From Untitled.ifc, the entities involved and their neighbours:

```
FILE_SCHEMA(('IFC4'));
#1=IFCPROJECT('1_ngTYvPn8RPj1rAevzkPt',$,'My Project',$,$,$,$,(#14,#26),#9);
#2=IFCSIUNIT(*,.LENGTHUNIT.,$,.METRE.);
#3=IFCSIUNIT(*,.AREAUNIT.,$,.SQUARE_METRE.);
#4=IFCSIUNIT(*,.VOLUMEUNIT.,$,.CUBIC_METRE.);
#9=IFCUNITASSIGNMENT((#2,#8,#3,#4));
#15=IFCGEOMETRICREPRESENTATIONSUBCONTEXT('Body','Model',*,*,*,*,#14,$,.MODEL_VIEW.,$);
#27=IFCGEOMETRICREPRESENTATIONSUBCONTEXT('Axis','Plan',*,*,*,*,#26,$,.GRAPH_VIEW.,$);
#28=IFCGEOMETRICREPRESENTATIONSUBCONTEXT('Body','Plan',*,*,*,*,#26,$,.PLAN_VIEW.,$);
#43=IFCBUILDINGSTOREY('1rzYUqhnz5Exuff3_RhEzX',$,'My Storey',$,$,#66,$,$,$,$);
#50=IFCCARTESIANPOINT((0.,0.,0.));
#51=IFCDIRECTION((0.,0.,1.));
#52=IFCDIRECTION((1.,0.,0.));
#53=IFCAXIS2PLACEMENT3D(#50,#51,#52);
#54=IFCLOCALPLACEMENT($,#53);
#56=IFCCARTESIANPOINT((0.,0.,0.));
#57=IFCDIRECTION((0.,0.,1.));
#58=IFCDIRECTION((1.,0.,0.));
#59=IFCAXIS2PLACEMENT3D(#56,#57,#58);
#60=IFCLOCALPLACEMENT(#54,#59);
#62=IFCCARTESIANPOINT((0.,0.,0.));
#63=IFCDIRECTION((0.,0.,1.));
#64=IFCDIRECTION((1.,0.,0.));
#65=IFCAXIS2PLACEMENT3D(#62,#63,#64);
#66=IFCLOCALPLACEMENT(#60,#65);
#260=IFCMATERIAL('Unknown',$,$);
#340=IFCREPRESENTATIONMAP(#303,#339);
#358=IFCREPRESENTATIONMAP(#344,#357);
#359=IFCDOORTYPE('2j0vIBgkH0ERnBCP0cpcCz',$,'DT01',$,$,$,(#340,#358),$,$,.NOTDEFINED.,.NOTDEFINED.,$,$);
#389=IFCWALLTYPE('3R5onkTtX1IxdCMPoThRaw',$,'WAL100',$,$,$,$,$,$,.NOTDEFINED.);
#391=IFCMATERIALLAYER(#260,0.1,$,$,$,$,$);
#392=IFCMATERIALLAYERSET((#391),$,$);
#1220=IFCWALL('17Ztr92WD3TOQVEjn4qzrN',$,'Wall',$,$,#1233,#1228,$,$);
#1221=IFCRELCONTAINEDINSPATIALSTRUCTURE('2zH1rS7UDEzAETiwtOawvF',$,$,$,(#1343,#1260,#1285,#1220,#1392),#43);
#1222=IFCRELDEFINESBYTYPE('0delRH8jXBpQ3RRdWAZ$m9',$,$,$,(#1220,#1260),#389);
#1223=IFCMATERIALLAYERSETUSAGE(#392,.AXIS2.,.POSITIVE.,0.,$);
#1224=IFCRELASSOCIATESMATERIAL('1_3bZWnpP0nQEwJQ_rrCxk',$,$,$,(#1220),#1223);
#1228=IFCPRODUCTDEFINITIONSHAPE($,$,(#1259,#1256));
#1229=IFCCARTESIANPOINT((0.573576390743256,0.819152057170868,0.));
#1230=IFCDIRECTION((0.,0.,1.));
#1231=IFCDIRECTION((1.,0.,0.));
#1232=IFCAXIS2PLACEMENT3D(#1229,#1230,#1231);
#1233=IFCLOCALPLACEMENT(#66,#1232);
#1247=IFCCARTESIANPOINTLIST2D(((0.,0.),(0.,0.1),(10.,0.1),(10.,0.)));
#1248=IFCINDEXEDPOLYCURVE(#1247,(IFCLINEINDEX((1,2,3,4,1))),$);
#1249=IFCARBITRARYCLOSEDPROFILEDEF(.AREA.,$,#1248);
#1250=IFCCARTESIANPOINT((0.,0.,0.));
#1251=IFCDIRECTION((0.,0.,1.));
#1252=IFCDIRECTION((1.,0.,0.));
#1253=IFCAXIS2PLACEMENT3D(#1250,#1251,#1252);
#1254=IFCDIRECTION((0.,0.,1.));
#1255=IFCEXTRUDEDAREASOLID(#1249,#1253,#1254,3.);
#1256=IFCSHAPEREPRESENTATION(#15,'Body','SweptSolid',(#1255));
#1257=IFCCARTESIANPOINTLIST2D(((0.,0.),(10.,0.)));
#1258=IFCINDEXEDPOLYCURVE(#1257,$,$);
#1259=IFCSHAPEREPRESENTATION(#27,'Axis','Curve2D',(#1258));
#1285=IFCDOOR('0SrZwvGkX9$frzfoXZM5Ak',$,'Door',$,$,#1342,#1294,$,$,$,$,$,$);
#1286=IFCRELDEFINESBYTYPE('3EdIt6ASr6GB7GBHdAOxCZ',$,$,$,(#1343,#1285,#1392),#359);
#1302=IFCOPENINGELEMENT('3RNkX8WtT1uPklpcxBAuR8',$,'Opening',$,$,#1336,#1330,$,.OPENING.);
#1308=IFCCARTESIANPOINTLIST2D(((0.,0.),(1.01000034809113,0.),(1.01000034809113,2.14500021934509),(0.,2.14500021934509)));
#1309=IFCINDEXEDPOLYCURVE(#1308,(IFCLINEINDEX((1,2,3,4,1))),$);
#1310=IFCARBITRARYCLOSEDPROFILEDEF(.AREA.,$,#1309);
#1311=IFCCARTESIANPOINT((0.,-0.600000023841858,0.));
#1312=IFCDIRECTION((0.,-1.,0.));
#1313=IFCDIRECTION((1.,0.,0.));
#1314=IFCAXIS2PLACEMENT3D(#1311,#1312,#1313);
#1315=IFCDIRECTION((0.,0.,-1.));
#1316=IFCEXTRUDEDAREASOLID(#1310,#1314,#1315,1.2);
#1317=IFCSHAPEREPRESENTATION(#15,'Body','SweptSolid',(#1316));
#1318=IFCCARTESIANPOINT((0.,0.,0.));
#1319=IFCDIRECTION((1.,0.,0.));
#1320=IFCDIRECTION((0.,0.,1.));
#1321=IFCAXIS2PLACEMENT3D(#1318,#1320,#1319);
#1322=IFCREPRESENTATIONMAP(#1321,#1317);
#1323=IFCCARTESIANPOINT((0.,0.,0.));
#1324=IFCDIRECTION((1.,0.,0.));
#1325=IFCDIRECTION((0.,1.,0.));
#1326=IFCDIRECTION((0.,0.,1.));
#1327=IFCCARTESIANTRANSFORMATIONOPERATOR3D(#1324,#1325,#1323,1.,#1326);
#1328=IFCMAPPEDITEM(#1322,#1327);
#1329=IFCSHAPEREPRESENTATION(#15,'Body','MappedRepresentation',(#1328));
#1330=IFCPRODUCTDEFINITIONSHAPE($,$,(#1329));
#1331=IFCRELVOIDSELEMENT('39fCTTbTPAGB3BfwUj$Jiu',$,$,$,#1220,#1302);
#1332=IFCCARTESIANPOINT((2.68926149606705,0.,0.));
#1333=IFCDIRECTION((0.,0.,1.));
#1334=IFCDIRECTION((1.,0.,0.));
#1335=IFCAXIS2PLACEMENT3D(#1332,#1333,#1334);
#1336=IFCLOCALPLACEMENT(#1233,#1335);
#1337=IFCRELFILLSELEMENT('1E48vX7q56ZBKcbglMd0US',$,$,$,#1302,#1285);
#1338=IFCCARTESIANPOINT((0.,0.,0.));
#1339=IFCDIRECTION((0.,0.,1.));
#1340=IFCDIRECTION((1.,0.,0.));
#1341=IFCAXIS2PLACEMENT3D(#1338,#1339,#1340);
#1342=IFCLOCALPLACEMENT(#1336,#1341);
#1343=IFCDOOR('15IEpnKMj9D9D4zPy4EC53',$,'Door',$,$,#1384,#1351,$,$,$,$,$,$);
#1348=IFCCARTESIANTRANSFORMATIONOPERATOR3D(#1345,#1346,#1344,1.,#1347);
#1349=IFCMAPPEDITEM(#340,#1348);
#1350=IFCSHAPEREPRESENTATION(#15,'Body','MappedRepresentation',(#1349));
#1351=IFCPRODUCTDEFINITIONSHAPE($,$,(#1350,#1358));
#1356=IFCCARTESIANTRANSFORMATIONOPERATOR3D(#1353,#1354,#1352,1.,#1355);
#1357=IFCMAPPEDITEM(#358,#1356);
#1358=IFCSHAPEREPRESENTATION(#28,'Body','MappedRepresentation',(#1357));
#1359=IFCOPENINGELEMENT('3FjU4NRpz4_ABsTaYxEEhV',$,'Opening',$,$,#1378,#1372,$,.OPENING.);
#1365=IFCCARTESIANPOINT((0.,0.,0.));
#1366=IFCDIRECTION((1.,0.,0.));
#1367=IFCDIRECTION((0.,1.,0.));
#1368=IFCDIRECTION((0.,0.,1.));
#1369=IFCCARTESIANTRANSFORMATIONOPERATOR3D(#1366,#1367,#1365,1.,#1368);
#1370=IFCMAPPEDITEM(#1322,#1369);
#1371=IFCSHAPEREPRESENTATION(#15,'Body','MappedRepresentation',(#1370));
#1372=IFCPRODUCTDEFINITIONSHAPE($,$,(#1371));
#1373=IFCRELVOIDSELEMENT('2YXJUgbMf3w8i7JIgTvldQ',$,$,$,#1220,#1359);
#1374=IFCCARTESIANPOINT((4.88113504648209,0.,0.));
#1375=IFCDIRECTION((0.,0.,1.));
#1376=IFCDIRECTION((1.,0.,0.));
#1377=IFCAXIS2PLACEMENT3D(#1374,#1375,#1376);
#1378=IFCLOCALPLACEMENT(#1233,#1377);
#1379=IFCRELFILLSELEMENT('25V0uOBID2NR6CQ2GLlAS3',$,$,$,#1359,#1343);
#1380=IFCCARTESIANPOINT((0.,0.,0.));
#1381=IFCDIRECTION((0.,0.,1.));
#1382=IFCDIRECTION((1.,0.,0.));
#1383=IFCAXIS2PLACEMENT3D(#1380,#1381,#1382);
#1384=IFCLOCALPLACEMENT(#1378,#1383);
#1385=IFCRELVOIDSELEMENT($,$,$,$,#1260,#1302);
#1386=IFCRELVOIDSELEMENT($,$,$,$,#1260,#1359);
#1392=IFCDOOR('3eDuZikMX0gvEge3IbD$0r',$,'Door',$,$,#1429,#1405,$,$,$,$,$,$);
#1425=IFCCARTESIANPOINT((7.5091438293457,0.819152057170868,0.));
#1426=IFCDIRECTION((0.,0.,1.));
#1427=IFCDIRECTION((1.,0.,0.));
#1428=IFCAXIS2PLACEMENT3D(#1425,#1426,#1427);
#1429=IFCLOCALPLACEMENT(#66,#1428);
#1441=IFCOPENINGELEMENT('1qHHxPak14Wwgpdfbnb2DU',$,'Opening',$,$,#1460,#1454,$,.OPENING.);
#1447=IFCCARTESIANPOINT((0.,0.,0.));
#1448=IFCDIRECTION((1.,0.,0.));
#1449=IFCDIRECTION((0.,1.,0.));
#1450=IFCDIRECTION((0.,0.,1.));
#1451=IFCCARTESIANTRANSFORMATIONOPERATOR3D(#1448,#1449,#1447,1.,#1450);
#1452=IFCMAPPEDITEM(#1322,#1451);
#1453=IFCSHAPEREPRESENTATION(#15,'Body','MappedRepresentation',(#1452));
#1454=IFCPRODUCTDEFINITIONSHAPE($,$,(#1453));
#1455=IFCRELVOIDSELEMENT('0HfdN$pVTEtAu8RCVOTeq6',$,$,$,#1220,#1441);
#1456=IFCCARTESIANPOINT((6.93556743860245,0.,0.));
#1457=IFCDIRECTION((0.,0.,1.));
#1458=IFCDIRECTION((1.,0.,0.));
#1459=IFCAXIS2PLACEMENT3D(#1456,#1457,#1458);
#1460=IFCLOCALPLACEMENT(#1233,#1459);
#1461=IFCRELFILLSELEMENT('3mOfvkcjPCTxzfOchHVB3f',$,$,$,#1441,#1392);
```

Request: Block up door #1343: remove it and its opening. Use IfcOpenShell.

```python
import ifcopenshell
import ifcopenshell.api.feature
import ifcopenshell.api.root
import ifcopenshell.geom
import ifcopenshell.util.shape

model = ifcopenshell.open("Untitled.ifc")
settings = ifcopenshell.geom.settings()


def volume(element):
    """Net volume in cubic metres, openings subtracted."""
    shape = ifcopenshell.geom.create_shape(settings, element)
    return ifcopenshell.util.shape.get_volume(shape.geometry)


door = model.by_id(1343)
opening = door.FillsVoids[0].RelatingOpeningElement
wall = opening.VoidsElements[0].RelatingBuildingElement
before = volume(wall)

ifcopenshell.api.root.remove_product(model, product=door)
ifcopenshell.api.feature.remove_feature(model, feature=opening)

after = volume(wall)

print(f"wall volume {before:.3f} -> {after:.3f} m3")

model.write("Untitled_updated.ifc")
```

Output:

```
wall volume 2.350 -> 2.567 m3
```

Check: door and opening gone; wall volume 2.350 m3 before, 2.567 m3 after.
